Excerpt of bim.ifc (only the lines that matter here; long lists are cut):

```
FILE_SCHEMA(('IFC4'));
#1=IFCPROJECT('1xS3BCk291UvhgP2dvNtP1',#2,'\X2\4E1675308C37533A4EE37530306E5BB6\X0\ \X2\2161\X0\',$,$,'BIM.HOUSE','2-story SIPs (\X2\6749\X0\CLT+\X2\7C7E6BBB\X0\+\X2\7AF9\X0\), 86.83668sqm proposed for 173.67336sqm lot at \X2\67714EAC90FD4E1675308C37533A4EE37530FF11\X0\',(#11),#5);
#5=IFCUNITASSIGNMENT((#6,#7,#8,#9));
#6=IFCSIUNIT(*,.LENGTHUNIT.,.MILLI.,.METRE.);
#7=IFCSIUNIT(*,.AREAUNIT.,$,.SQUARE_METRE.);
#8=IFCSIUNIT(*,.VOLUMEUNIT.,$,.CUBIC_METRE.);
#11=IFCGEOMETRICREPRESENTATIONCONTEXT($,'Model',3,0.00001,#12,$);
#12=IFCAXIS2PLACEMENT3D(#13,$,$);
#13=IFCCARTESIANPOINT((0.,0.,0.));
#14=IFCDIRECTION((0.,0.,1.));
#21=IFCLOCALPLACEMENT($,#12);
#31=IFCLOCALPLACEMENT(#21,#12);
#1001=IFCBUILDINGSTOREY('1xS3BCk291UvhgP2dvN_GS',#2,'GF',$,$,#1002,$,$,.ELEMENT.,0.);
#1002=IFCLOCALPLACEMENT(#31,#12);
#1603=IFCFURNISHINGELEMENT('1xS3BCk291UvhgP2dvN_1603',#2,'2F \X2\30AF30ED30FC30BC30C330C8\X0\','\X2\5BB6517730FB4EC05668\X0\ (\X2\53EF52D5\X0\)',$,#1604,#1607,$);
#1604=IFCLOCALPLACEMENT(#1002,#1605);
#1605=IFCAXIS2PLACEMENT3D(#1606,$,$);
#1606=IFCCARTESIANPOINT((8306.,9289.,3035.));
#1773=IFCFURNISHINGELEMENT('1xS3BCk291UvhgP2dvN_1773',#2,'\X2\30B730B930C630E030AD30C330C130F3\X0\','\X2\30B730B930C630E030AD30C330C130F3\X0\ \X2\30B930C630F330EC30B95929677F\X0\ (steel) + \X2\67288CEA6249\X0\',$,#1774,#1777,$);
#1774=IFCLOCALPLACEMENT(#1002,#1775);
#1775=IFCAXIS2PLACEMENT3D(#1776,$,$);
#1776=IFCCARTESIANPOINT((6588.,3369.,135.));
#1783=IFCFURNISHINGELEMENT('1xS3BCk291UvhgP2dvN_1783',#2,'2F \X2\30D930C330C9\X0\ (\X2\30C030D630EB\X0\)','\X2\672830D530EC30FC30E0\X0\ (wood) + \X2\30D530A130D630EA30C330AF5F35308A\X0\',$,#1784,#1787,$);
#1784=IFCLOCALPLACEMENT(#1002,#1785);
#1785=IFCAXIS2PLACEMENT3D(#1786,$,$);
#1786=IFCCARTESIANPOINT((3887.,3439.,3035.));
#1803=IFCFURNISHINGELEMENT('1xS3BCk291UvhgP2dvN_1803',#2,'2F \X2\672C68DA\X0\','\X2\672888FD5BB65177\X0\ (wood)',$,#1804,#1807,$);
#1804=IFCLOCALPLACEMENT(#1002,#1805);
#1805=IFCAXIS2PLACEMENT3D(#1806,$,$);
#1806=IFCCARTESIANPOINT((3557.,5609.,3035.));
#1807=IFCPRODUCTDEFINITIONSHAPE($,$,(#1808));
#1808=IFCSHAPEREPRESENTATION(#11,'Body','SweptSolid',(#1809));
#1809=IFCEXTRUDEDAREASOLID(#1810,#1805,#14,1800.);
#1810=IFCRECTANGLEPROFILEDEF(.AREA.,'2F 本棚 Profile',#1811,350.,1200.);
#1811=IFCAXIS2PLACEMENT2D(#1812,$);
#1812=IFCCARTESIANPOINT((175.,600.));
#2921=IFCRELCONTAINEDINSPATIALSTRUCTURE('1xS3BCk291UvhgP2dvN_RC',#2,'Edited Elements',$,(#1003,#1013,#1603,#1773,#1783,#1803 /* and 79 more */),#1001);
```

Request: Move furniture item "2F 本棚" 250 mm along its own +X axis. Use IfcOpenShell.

```python
import ifcopenshell
import ifcopenshell.api.geometry
import ifcopenshell.util.placement

model = ifcopenshell.open("bim.ifc")

item = model.by_guid("1xS3BCk291UvhgP2dvN_1803")
matrix = ifcopenshell.util.placement.get_local_placement(item.ObjectPlacement)
matrix[:3, 3] += matrix[:3, 0] * 250.0
ifcopenshell.api.geometry.edit_object_placement(model, product=item, matrix=matrix, is_si=False)

print(ifcopenshell.util.placement.get_local_placement(item.ObjectPlacement).round(3) + 0.0)

model.write("bim_edited.ifc")
```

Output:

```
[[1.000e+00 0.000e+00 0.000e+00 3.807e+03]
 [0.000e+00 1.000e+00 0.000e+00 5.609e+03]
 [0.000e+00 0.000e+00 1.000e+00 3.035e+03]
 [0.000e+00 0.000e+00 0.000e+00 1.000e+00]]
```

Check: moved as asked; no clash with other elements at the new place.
